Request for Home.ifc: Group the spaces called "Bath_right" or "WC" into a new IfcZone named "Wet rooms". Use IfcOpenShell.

First a look at what the model holds.

```python
import ifcopenshell

model = ifcopenshell.open("Home.ifc")
print(model.schema)
seen = {}
for space in model.by_type("IfcSpace"):
    seen[space.LongName] = seen.get(space.LongName, 0) + 1
for name, count in sorted(seen.items(), key=str):
    print(count, "x", name)
print("zones:", [z.Name for z in model.by_type("IfcZone")][:20])
```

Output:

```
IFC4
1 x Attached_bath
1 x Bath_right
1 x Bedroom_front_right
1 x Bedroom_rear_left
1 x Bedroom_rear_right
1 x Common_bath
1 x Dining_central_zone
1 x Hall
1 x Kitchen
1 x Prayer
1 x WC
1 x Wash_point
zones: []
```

```python
import ifcopenshell
import ifcopenshell.api.group
import ifcopenshell.api.root

model = ifcopenshell.open("Home.ifc")

names = {"Bath_right", "WC"}
spaces = [s for s in model.by_type("IfcSpace") if s.LongName in names]

zone = ifcopenshell.api.root.create_entity(model, ifc_class="IfcZone", name="Wet rooms")
ifcopenshell.api.group.assign_group(model, products=spaces, group=zone)
print(len(spaces), "spaces in", zone.Name)

model.write("Home-out.ifc")
```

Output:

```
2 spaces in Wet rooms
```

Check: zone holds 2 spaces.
